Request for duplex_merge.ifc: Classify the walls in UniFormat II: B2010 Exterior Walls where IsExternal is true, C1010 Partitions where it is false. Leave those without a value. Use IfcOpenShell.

First a look at what the model holds.

```python
import ifcopenshell
import ifcopenshell.util.element

model = ifcopenshell.open("duplex_merge.ifc")
print(model.schema)
print("classifications:", [c.Name for c in model.by_type("IfcClassification")])
values = [ifcopenshell.util.element.get_pset(e, "Pset_WallCommon", "IsExternal") for e in model.by_type("IfcWall")]
for value in (True, False, None):
    print("IsExternal", value, values.count(value))
```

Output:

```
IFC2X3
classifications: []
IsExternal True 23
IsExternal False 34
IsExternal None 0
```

```python
import ifcopenshell
import ifcopenshell.api.classification
import ifcopenshell.util.element

model = ifcopenshell.open("duplex_merge.ifc")

# IFC2X3 requires Source and Edition and has no link from the project to the system.
system = model.create_entity("IfcClassification", Source="ASTM", Edition="E1557", Name="UniFormat II")

walls = model.by_type("IfcWall")
external = {e: ifcopenshell.util.element.get_pset(e, "Pset_WallCommon", "IsExternal") for e in walls}
for flag, code, name in ((True, "B2010", "Exterior Walls"), (False, "C1010", "Partitions")):
    products = [e for e in walls if external[e] is flag]
    ifcopenshell.api.classification.add_reference(
        model, products=products, classification=system, identification=code, name=name
    )
    print(code, len(products))

model.write("duplex_merge_rev.ifc")
```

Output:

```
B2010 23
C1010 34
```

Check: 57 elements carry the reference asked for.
